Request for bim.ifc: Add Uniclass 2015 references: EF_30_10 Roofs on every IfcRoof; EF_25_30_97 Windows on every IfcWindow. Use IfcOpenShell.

First a look at what the model holds.

```python
import ifcopenshell

model = ifcopenshell.open("bim.ifc")
print(model.schema)
print("classifications:", [c.Name for c in model.by_type("IfcClassification")])
for ifc_class in ("IfcDoor", "IfcRoof", "IfcStair", "IfcWall", "IfcWindow"):
    print(ifc_class, len(model.by_type(ifc_class)))
```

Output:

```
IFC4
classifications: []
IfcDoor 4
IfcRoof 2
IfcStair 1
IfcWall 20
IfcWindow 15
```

```python
import ifcopenshell
import ifcopenshell.api.classification

model = ifcopenshell.open("bim.ifc")

system = ifcopenshell.api.classification.add_classification(model, classification="Uniclass 2015")

codes = {
    "IfcRoof": ("EF_30_10", "Roofs"),
    "IfcWindow": ("EF_25_30_97", "Windows"),
}
for ifc_class, (code, name) in codes.items():
    products = model.by_type(ifc_class)
    ifcopenshell.api.classification.add_reference(
        model, products=products, classification=system, identification=code, name=name
    )
    print(code, len(products))

model.write("bim_v2.ifc")
```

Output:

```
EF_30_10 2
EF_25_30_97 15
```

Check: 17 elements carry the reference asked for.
